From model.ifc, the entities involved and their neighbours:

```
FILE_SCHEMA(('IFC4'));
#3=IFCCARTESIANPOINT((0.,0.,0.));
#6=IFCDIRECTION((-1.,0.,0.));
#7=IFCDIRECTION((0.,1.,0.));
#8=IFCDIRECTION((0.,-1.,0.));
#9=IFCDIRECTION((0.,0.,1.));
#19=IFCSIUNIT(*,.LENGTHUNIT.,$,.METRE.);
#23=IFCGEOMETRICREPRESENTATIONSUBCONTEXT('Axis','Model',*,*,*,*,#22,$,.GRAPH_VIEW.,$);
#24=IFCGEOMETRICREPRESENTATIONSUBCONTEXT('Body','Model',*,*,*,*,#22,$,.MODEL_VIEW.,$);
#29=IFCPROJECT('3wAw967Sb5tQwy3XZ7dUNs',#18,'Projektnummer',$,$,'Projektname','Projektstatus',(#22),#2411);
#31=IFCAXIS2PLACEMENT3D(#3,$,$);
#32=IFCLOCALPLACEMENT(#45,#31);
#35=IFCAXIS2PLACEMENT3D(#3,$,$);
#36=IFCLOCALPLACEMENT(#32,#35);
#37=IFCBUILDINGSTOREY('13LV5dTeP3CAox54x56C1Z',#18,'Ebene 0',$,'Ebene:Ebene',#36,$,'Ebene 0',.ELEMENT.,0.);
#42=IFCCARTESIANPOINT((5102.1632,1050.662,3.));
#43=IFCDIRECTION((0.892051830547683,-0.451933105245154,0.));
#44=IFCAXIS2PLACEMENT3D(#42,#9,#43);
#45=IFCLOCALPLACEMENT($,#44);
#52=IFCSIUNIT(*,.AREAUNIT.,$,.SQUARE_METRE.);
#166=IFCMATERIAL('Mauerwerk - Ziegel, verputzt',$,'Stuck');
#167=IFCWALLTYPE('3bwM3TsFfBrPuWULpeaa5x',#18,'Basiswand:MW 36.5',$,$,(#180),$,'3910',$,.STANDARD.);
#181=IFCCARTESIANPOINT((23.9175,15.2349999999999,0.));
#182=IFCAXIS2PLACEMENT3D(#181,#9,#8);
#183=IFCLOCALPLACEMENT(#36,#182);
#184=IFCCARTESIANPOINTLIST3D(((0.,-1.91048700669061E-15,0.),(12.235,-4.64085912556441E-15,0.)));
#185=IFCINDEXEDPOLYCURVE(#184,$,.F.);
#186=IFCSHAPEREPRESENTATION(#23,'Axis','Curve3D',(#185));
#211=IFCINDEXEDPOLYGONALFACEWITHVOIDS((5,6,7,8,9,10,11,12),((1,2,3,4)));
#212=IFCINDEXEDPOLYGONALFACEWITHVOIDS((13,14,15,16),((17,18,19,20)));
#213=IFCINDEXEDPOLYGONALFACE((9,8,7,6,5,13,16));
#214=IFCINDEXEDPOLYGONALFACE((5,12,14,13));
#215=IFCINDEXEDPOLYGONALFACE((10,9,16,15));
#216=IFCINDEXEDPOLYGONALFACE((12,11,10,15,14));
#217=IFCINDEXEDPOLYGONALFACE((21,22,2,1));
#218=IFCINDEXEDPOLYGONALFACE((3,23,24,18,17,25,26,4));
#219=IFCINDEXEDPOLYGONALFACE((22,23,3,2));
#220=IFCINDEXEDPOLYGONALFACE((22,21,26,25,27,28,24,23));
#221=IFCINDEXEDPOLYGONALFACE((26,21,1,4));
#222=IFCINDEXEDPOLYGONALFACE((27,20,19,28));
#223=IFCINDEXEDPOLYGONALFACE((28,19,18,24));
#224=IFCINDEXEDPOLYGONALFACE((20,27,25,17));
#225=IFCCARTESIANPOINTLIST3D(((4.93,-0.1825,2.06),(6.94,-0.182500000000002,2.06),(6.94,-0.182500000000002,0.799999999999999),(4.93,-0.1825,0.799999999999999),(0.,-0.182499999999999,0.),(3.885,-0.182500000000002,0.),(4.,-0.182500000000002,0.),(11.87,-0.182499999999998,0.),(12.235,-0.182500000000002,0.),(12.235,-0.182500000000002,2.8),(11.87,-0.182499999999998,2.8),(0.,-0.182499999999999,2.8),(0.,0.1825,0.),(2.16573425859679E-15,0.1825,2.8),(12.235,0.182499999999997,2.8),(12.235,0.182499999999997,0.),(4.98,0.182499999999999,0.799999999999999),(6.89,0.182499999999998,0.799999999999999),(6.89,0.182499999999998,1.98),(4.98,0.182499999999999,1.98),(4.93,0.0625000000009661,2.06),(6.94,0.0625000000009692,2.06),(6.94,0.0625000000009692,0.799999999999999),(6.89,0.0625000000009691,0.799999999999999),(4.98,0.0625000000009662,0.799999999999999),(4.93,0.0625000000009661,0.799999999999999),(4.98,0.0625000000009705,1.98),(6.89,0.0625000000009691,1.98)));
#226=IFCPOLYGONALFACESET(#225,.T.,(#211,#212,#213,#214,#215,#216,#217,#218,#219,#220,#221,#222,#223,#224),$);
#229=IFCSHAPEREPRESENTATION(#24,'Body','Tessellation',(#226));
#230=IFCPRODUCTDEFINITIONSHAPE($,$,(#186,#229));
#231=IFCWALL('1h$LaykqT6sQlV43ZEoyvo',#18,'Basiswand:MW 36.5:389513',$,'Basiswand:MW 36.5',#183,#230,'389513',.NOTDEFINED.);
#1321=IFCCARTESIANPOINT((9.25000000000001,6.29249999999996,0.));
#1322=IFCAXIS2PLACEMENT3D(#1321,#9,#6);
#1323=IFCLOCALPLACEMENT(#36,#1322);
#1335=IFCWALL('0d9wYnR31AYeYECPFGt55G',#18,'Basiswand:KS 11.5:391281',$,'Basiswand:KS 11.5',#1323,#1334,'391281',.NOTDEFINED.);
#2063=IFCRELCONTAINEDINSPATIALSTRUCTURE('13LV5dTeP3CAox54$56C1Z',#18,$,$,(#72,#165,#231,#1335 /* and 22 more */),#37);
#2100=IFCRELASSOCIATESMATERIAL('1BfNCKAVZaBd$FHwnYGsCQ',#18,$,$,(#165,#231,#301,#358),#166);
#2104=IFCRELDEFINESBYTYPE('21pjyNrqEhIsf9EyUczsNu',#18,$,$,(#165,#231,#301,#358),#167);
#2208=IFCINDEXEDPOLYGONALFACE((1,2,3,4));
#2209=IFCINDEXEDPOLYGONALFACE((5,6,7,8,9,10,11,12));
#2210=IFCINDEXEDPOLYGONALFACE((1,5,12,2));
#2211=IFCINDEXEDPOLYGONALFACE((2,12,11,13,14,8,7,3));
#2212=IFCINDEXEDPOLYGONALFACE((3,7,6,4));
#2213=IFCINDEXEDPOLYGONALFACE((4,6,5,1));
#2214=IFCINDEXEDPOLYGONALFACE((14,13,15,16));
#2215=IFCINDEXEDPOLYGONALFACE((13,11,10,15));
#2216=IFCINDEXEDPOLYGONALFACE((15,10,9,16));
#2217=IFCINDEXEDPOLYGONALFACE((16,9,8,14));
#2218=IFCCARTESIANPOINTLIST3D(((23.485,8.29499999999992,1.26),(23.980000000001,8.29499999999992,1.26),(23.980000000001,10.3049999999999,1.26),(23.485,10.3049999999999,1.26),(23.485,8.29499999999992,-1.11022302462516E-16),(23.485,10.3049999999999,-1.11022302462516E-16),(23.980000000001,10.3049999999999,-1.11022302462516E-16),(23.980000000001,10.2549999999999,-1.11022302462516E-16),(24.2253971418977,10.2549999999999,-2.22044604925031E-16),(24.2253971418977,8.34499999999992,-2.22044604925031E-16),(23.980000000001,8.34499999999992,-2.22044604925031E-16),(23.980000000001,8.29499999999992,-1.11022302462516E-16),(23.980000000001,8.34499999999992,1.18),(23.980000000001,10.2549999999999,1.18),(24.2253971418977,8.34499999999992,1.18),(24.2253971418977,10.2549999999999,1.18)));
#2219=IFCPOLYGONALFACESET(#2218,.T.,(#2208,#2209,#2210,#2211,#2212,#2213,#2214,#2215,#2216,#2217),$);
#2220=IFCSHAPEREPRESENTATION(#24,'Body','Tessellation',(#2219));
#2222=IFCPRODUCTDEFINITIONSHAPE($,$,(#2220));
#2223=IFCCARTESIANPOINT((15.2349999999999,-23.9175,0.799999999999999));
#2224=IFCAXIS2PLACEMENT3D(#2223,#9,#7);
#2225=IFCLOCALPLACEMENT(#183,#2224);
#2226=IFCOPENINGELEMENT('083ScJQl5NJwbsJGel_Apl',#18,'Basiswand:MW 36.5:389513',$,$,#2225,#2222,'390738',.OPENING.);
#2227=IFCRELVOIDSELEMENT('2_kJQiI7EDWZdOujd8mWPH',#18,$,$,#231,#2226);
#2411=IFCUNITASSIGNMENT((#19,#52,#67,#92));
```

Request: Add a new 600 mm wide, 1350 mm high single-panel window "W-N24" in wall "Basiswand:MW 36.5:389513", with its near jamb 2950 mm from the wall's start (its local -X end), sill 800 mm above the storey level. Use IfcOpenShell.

```python
import numpy as np
import ifcopenshell
import ifcopenshell.api.feature
import ifcopenshell.api.geometry
import ifcopenshell.api.root
import ifcopenshell.api.spatial
import ifcopenshell.geom
import ifcopenshell.util.element
import ifcopenshell.util.placement
import ifcopenshell.util.representation
import ifcopenshell.util.shape
import ifcopenshell.util.unit

model = ifcopenshell.open("model.ifc")
unit_scale = ifcopenshell.util.unit.calculate_unit_scale(model)
settings = ifcopenshell.geom.settings()


def volume(element):
    """Net volume in cubic metres, openings subtracted."""
    shape = ifcopenshell.geom.create_shape(settings, element)
    return ifcopenshell.util.shape.get_volume(shape.geometry)


wall = model.by_id(231)
storey = ifcopenshell.util.element.get_container(wall, ifc_class="IfcBuildingStorey")
context = ifcopenshell.util.representation.get_context(model, "Model", "Body", "MODEL_VIEW")
before = volume(wall)

width, height, from_end, sill = 0.6, 1.35, 2.95, 0.8  # metres

# The wall runs along its own X axis, and the end named is its -X end.
wall_shape = ifcopenshell.geom.create_shape(settings, wall)
x, y, z = ifcopenshell.util.shape.get_vertices(wall_shape.geometry).T
start = x.min() + from_end
face, thickness = float(y.min()), float(y.max() - y.min())
wall_matrix = ifcopenshell.util.placement.get_local_placement(wall.ObjectPlacement)
level = ifcopenshell.util.placement.get_local_placement(storey.ObjectPlacement)[2, 3]


def in_wall(x, y):
    """Placement at x, y metres in the wall's axes, at sill height."""
    matrix = wall_matrix.copy()
    matrix[:, 3] = wall_matrix @ np.array([x / unit_scale, y / unit_scale, 0.0, 1.0])
    matrix[2, 3] = level + sill / unit_scale
    return matrix


# Opening: a box that overshoots both wall faces by 50 mm.
opening = ifcopenshell.api.root.create_entity(model, ifc_class="IfcOpeningElement", predefined_type="OPENING")
box = ifcopenshell.api.geometry.add_wall_representation(
    model, context=context, length=width, height=height, thickness=thickness + 0.1
)
ifcopenshell.api.geometry.assign_representation(model, product=opening, representation=box)
ifcopenshell.api.geometry.edit_object_placement(model, product=opening, matrix=in_wall(start, face - 0.05), is_si=False)
ifcopenshell.api.feature.add_feature(model, feature=opening, element=wall)

window = ifcopenshell.api.root.create_entity(model, ifc_class="IfcWindow", name="W-N24", predefined_type="WINDOW")
window.OverallWidth, window.OverallHeight = width / unit_scale, height / unit_scale
window.PartitioningType = "SINGLE_PANEL"
body = ifcopenshell.api.geometry.add_window_representation(
    model,
    context=context,
    overall_width=window.OverallWidth,
    overall_height=window.OverallHeight,
    partition_type="SINGLE_PANEL",
)
ifcopenshell.api.geometry.assign_representation(model, product=window, representation=body)
ifcopenshell.api.spatial.assign_container(model, products=[window], relating_structure=storey)
ifcopenshell.api.feature.add_filling(model, opening=opening, element=window)

# Centre the window in the wall's thickness.
ifcopenshell.api.geometry.edit_object_placement(model, product=window, matrix=in_wall(start, face), is_si=False)
window_shape = ifcopenshell.geom.create_shape(settings, window)
depth = ifcopenshell.util.shape.get_vertices(window_shape.geometry)[:, 1]
offset = face + thickness / 2 - (depth.min() + depth.max()) / 2
ifcopenshell.api.geometry.edit_object_placement(model, product=window, matrix=in_wall(start, offset), is_si=False)

after = volume(wall)

print(f"wall volume {before:.3f} -> {after:.3f} m3")

model.write("model_rev.ifc")
```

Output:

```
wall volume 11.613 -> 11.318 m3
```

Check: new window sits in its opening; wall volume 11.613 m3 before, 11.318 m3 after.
